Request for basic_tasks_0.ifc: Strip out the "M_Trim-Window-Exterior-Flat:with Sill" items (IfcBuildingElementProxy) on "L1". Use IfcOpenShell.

First a look at what the model holds.

```python
import ifcopenshell
import ifcopenshell.util.element

model = ifcopenshell.open("basic_tasks_0.ifc")
print(model.schema)
storey = next(s for s in model.by_type("IfcBuildingStorey") if s.Name == "L1")
proxies = [e for e in ifcopenshell.util.element.get_decomposition(storey) if e.is_a("IfcBuildingElementProxy")]
seen = {}
for e in proxies:
    element_type = ifcopenshell.util.element.get_type(e)
    name = element_type.Name if element_type not in (None, e) else None
    seen[name] = seen.get(name, 0) + 1
for name, count in sorted(seen.items(), key=str):
    print(count, "x", name)
```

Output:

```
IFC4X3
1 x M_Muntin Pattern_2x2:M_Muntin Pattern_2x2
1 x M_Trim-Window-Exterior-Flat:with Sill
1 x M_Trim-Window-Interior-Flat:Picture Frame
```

```python
import ifcopenshell
import ifcopenshell.api.root
import ifcopenshell.util.element

model = ifcopenshell.open("basic_tasks_0.ifc")

storey = next(s for s in model.by_type("IfcBuildingStorey") if s.Name == "L1")
proxies = [e for e in ifcopenshell.util.element.get_decomposition(storey) if e.is_a("IfcBuildingElementProxy")]
targets = [e for e in proxies if (t := ifcopenshell.util.element.get_type(e)) not in (None, e) and t.Name == "M_Trim-Window-Exterior-Flat:with Sill"]

for e in targets:
    ifcopenshell.api.root.remove_product(model, product=e)
print(len(targets), "removed")

model.write("basic_tasks_0_edited.ifc")
```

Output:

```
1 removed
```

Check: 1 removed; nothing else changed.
